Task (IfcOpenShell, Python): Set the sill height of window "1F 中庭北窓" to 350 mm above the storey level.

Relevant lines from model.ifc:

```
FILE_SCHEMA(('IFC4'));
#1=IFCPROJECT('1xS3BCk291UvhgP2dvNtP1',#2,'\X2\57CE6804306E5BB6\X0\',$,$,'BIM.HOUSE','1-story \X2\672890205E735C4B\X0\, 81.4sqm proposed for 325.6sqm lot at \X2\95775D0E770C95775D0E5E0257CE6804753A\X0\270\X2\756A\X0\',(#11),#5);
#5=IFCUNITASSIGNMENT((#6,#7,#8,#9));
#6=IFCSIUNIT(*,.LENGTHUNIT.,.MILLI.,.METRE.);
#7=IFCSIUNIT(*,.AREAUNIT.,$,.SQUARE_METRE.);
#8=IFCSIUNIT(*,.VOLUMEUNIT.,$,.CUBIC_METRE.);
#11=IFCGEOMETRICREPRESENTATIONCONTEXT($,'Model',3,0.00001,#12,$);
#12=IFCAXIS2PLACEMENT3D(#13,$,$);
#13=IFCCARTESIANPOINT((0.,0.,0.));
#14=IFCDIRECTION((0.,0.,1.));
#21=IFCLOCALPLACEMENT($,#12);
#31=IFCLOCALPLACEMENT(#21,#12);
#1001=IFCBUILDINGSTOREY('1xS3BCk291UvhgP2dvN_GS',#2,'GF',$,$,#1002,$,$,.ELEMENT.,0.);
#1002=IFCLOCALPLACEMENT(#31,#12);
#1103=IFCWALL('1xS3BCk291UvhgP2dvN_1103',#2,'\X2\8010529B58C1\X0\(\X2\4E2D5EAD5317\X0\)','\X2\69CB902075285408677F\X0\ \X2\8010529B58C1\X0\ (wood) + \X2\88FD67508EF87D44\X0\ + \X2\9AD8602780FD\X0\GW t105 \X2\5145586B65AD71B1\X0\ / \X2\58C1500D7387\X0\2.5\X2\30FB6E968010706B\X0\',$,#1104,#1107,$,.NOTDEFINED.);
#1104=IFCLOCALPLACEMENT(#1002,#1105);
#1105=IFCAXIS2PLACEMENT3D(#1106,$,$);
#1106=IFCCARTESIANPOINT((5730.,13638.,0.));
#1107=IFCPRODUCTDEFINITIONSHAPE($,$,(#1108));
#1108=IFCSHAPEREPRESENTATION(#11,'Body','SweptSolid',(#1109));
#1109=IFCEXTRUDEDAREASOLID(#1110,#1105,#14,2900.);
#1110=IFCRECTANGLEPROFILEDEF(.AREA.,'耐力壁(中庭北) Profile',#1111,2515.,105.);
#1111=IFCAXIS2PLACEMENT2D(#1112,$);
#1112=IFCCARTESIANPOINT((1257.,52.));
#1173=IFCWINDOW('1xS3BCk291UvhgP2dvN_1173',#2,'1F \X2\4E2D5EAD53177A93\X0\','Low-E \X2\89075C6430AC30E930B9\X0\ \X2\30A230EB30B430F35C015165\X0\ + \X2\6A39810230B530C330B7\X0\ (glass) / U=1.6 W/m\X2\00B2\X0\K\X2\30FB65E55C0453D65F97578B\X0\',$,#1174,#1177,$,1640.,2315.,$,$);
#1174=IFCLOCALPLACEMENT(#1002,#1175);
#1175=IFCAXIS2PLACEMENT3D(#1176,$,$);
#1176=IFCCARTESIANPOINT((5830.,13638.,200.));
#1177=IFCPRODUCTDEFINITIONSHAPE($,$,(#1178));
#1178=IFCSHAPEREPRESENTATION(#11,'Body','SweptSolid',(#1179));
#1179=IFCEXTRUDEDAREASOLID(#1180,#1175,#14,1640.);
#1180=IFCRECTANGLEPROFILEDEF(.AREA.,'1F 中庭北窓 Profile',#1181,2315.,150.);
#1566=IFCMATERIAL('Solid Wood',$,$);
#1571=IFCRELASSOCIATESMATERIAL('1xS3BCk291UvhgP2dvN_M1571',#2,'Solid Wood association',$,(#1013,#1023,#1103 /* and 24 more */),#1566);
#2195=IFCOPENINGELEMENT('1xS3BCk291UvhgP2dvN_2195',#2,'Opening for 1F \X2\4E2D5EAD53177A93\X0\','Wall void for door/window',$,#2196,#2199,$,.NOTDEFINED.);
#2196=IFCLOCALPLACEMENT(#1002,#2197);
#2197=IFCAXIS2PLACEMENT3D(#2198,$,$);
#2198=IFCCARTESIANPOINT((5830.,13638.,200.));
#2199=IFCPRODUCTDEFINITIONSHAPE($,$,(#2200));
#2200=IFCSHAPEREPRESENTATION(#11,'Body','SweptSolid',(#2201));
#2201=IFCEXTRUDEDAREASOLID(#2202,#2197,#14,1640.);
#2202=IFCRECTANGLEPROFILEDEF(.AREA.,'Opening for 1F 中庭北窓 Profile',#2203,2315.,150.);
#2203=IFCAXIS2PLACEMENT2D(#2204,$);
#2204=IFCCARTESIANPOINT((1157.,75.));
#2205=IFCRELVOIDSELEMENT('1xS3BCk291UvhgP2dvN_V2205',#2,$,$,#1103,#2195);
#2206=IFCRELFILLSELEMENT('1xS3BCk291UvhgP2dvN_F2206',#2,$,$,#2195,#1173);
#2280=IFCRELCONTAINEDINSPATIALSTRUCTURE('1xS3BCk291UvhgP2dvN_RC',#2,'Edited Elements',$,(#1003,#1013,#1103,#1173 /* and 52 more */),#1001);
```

```python
import numpy as np
import ifcopenshell
import ifcopenshell.api.geometry
import ifcopenshell.geom
import ifcopenshell.util.element
import ifcopenshell.util.placement
import ifcopenshell.util.shape
import ifcopenshell.util.unit

model = ifcopenshell.open("model.ifc")
unit_scale = ifcopenshell.util.unit.calculate_unit_scale(model)

window = model.by_id(1173)
opening = window.FillsVoids[0].RelatingOpeningElement
storey = ifcopenshell.util.element.get_container(window, ifc_class="IfcBuildingStorey")
level = ifcopenshell.util.placement.get_local_placement(storey.ObjectPlacement)[2, 3]

# The opening's origin need not be at the sill, so measure its lowest point.
shape = ifcopenshell.geom.create_shape(ifcopenshell.geom.settings(), opening)
bottom = ifcopenshell.util.shape.get_shape_bottom_elevation(shape, shape.geometry) / unit_scale
dz = level + 350.0 - bottom

shift = np.array([0.0, 0.0, dz])
# The window is not placed relative to its opening, so move both.
for product in (opening, window):
    matrix = ifcopenshell.util.placement.get_local_placement(product.ObjectPlacement)
    matrix[:3, 3] += shift
    ifcopenshell.api.geometry.edit_object_placement(model, product=product, matrix=matrix, is_si=False)

print(f"moved by {dz * unit_scale:+.3f} m")

model.write("model_v2.ifc")
```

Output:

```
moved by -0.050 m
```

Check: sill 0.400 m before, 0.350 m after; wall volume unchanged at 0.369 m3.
